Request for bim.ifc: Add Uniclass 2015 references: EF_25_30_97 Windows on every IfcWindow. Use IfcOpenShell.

First a look at what the model holds.

```python
import ifcopenshell

model = ifcopenshell.open("bim.ifc")
print(model.schema)
print("classifications:", [c.Name for c in model.by_type("IfcClassification")])
for ifc_class in ("IfcDoor", "IfcRoof", "IfcStair", "IfcWall", "IfcWindow"):
    print(ifc_class, len(model.by_type(ifc_class)))
```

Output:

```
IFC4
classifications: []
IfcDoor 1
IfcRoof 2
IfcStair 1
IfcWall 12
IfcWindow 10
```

```python
import ifcopenshell
import ifcopenshell.api.classification

model = ifcopenshell.open("bim.ifc")

system = ifcopenshell.api.classification.add_classification(model, classification="Uniclass 2015")

codes = {
    "IfcWindow": ("EF_25_30_97", "Windows"),
}
for ifc_class, (code, name) in codes.items():
    products = model.by_type(ifc_class)
    ifcopenshell.api.classification.add_reference(
        model, products=products, classification=system, identification=code, name=name
    )
    print(code, len(products))

model.write("bim_v2.ifc")
```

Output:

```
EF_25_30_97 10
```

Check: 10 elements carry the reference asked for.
